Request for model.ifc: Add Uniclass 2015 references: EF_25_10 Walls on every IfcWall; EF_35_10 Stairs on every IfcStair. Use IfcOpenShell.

First a look at what the model holds.

```python
import ifcopenshell

model = ifcopenshell.open("model.ifc")
print(model.schema)
print("classifications:", [c.Name for c in model.by_type("IfcClassification")])
for ifc_class in ("IfcDoor", "IfcRoof", "IfcStair", "IfcWall", "IfcWindow"):
    print(ifc_class, len(model.by_type(ifc_class)))
```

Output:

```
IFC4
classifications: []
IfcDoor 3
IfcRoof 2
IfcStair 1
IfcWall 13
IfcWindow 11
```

```python
import ifcopenshell
import ifcopenshell.api.classification

model = ifcopenshell.open("model.ifc")

system = ifcopenshell.api.classification.add_classification(model, classification="Uniclass 2015")

codes = {
    "IfcWall": ("EF_25_10", "Walls"),
    "IfcStair": ("EF_35_10", "Stairs"),
}
for ifc_class, (code, name) in codes.items():
    products = model.by_type(ifc_class)
    ifcopenshell.api.classification.add_reference(
        model, products=products, classification=system, identification=code, name=name
    )
    print(code, len(products))

model.write("model_edited.ifc")
```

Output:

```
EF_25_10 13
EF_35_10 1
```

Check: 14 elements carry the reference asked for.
